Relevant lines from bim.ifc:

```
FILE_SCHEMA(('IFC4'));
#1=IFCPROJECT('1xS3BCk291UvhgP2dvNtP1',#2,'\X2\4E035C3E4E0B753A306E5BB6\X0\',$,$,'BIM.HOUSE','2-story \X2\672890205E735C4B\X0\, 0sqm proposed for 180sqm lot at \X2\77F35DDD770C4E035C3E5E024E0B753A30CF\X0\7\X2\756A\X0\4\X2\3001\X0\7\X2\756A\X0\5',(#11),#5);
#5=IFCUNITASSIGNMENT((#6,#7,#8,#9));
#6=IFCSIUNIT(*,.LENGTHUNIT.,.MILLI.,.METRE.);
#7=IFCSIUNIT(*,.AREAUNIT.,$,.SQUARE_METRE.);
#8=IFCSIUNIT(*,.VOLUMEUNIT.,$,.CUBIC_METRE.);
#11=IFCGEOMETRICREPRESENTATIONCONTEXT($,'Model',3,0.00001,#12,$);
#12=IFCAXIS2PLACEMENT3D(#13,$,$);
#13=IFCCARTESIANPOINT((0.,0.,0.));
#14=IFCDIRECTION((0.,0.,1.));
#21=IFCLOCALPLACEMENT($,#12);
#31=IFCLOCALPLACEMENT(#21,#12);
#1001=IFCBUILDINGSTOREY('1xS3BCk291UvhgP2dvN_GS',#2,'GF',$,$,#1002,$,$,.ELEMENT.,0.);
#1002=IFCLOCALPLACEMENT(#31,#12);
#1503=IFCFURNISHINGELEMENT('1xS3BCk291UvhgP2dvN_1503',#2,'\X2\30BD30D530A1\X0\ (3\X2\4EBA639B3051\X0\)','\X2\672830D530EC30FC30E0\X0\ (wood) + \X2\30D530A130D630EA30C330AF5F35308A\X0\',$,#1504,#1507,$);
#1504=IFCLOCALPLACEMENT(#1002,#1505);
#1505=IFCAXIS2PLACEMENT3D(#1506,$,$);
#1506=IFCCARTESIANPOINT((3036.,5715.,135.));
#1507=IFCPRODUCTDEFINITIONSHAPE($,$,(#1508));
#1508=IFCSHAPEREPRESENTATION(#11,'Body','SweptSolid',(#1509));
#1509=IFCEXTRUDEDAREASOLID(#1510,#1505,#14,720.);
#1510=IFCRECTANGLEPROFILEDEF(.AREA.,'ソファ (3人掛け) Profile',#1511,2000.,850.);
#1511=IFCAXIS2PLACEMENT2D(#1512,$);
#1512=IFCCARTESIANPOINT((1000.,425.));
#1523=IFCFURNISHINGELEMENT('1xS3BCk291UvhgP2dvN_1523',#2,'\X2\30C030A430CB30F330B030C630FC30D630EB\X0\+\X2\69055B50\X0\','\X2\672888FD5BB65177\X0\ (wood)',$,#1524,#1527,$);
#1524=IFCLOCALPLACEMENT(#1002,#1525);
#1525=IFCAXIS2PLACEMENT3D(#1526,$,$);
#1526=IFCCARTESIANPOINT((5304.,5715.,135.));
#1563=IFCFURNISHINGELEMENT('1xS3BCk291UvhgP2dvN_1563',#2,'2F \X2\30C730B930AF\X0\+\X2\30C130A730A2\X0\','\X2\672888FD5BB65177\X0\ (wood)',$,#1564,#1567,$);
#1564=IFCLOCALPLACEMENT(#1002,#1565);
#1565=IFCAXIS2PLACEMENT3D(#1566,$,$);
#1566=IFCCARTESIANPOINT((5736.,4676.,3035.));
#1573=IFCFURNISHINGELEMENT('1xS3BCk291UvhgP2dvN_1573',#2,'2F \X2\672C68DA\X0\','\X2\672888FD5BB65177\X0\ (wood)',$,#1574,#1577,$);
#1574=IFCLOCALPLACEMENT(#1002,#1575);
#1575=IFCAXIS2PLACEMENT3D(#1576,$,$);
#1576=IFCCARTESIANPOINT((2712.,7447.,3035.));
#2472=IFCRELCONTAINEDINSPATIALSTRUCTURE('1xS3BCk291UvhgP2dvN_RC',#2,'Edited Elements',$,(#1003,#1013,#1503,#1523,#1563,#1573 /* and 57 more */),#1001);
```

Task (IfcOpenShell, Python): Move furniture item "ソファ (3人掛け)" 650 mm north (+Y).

```python
import ifcopenshell
import ifcopenshell.api.geometry
import ifcopenshell.util.placement

model = ifcopenshell.open("bim.ifc")

item = model.by_guid("1xS3BCk291UvhgP2dvN_1503")
matrix = ifcopenshell.util.placement.get_local_placement(item.ObjectPlacement)
matrix[1, 3] += 650.0
ifcopenshell.api.geometry.edit_object_placement(model, product=item, matrix=matrix, is_si=False)

print(ifcopenshell.util.placement.get_local_placement(item.ObjectPlacement).round(3) + 0.0)

model.write("bim_edited.ifc")
```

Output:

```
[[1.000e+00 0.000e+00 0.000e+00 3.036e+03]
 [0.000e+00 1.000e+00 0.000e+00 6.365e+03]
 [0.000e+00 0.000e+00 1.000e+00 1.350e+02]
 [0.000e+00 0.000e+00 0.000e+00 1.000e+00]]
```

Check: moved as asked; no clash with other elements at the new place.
